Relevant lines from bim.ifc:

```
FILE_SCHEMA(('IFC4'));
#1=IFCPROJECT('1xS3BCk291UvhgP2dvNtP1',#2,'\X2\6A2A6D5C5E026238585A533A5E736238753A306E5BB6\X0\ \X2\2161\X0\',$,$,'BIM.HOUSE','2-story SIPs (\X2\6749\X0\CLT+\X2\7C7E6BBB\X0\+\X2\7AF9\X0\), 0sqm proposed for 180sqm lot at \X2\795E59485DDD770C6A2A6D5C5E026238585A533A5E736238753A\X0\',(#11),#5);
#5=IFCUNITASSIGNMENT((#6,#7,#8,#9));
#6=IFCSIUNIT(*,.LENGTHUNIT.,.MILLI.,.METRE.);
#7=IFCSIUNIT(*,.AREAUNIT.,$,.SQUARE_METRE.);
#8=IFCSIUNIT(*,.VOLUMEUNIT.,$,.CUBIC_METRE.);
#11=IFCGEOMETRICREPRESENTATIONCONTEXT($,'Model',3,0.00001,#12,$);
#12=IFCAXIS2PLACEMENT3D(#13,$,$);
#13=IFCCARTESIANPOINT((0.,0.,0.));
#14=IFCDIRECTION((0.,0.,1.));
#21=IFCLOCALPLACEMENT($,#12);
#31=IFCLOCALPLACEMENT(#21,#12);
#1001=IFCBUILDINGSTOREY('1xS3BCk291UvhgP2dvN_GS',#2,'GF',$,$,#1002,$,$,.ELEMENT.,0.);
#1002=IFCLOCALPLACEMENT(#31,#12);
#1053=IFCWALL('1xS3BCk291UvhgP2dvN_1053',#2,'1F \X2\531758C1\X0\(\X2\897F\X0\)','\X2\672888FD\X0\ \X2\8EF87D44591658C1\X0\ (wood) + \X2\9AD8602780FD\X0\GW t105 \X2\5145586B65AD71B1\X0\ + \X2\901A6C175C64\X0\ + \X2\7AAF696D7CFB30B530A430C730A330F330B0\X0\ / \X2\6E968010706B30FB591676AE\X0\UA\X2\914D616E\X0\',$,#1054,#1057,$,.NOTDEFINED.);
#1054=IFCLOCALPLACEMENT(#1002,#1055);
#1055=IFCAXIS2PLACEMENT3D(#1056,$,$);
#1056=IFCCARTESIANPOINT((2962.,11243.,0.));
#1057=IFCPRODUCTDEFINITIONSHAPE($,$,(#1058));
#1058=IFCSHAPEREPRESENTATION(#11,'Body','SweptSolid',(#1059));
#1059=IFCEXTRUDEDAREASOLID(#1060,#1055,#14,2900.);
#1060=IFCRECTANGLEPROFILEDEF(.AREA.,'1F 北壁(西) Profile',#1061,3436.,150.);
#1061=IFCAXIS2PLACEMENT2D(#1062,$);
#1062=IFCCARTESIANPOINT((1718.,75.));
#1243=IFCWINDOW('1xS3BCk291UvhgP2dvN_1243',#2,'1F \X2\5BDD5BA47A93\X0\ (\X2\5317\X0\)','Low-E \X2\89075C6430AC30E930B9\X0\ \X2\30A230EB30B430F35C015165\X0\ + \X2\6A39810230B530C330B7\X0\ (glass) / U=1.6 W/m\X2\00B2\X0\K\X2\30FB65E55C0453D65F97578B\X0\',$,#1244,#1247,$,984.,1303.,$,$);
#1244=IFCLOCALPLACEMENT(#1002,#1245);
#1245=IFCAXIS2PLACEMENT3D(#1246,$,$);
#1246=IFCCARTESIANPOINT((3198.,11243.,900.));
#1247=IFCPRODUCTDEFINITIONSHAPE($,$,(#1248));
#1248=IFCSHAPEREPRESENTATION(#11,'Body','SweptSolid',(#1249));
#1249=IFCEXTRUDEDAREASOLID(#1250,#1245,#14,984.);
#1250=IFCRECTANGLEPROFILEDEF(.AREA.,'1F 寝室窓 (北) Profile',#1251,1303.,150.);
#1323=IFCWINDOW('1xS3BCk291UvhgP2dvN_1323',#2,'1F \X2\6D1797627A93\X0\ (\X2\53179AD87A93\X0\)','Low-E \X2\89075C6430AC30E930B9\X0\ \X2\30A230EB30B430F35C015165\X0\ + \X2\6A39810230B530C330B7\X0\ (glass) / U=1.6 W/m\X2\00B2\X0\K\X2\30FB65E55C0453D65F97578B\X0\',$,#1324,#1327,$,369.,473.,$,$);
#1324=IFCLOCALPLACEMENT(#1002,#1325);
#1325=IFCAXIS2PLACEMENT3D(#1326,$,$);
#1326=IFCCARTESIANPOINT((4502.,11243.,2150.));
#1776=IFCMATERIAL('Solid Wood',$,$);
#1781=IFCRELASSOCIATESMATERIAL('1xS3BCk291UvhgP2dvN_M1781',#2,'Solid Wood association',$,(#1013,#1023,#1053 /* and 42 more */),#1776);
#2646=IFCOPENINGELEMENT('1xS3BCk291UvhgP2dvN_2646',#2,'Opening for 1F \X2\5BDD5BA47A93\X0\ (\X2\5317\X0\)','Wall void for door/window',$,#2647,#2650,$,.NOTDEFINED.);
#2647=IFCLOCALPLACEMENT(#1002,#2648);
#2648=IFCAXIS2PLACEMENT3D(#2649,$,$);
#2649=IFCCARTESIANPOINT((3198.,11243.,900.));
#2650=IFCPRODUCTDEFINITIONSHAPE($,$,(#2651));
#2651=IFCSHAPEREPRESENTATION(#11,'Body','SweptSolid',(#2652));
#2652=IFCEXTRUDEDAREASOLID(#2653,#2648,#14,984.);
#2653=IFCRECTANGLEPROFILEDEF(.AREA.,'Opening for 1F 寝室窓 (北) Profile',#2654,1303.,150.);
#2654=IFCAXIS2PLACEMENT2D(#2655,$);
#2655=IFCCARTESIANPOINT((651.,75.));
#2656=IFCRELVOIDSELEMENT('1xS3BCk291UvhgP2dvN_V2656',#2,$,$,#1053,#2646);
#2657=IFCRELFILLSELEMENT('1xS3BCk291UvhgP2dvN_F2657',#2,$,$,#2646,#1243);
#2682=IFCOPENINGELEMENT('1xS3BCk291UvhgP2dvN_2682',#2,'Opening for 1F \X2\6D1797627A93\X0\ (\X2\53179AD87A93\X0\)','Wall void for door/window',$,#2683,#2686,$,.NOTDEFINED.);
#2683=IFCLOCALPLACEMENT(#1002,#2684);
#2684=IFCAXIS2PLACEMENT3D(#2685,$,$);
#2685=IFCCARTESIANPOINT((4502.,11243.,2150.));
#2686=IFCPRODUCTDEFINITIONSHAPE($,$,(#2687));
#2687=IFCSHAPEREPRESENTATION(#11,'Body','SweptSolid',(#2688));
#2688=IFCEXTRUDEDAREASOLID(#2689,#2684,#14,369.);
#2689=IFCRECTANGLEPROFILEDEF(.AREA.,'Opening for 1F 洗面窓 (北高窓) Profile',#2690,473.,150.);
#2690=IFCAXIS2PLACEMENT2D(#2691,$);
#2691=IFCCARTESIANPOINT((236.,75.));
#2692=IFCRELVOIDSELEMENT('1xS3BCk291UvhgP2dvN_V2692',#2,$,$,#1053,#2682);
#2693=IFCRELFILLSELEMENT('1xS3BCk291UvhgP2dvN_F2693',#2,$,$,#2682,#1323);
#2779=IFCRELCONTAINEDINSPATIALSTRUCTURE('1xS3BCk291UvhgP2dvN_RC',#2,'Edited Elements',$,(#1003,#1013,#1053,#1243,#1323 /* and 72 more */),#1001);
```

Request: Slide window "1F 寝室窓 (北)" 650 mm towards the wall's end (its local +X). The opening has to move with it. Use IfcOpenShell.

```python
import ifcopenshell
import ifcopenshell.api.geometry
import ifcopenshell.util.placement

model = ifcopenshell.open("bim.ifc")

window = model.by_guid("1xS3BCk291UvhgP2dvN_1243")
opening = window.FillsVoids[0].RelatingOpeningElement
wall = opening.VoidsElements[0].RelatingBuildingElement

wall_matrix = ifcopenshell.util.placement.get_local_placement(wall.ObjectPlacement)
shift = wall_matrix[:3, 0] * 650.0
before = ifcopenshell.util.placement.get_local_placement(window.ObjectPlacement)[:3, 3].copy()

# The window is not placed relative to its opening, so move both.
for product in (opening, window):
    matrix = ifcopenshell.util.placement.get_local_placement(product.ObjectPlacement)
    matrix[:3, 3] += shift
    ifcopenshell.api.geometry.edit_object_placement(model, product=product, matrix=matrix, is_si=False)

after = ifcopenshell.util.placement.get_local_placement(window.ObjectPlacement)[:3, 3]
print("window moved by", (after - before).round(3) + 0.0)

model.write("bim-out.ifc")
```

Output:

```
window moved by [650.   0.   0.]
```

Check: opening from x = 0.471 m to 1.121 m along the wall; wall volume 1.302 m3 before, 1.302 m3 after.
